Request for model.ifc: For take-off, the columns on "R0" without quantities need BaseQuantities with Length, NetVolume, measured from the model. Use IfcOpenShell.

First a look at what the model holds.

```python
import ifcopenshell
import ifcopenshell.util.element
import ifcopenshell.util.unit

model = ifcopenshell.open("model.ifc")
print(model.schema)
for unit_type in ("LENGTHUNIT", "AREAUNIT", "VOLUMEUNIT"):
    print(unit_type, ifcopenshell.util.unit.calculate_unit_scale(model, unit_type))
storey = next(s for s in model.by_type("IfcBuildingStorey") if s.Name == "R0")
columns = [e for e in ifcopenshell.util.element.get_decomposition(storey) if e.is_a("IfcColumn")]
for e in sorted(columns, key=lambda e: e.id()):
    print(e.id(), e.is_a(), e.Name, list(ifcopenshell.util.element.get_psets(e, qtos_only=True)), sep=" | ")
```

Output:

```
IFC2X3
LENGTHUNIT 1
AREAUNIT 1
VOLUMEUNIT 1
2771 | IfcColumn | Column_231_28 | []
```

```python
import ifcopenshell
import ifcopenshell.api.pset
import ifcopenshell.geom
import ifcopenshell.util.element
import ifcopenshell.util.shape
import ifcopenshell.util.unit

model = ifcopenshell.open("model.ifc")
unit_scale = ifcopenshell.util.unit.calculate_unit_scale(model)
volume_scale = ifcopenshell.util.unit.calculate_unit_scale(model, "VOLUMEUNIT")
settings = ifcopenshell.geom.settings()

storey = next(s for s in model.by_type("IfcBuildingStorey") if s.Name == "R0")
columns = [e for e in ifcopenshell.util.element.get_decomposition(storey) if e.is_a("IfcColumn")]

for e in sorted(columns, key=lambda e: e.id()):
    if ifcopenshell.util.element.get_psets(e, qtos_only=True, should_inherit=False):
        continue
    # Geometry comes back in metres, in the element's own axes.
    shape = ifcopenshell.geom.create_shape(settings, e)
    values = {
        "Length": ifcopenshell.util.shape.get_z(shape.geometry) / unit_scale,
        "NetVolume": ifcopenshell.util.shape.get_volume(shape.geometry) / volume_scale,
    }
    qto = ifcopenshell.api.pset.add_qto(model, product=e, name="BaseQuantities")
    ifcopenshell.api.pset.edit_qto(model, qto=qto, properties=values)
    print(e.id(), {k: round(v, 3) for k, v in values.items()})

model.write("model-out.ifc")
```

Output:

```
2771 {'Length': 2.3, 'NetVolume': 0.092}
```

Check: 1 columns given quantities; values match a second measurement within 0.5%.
